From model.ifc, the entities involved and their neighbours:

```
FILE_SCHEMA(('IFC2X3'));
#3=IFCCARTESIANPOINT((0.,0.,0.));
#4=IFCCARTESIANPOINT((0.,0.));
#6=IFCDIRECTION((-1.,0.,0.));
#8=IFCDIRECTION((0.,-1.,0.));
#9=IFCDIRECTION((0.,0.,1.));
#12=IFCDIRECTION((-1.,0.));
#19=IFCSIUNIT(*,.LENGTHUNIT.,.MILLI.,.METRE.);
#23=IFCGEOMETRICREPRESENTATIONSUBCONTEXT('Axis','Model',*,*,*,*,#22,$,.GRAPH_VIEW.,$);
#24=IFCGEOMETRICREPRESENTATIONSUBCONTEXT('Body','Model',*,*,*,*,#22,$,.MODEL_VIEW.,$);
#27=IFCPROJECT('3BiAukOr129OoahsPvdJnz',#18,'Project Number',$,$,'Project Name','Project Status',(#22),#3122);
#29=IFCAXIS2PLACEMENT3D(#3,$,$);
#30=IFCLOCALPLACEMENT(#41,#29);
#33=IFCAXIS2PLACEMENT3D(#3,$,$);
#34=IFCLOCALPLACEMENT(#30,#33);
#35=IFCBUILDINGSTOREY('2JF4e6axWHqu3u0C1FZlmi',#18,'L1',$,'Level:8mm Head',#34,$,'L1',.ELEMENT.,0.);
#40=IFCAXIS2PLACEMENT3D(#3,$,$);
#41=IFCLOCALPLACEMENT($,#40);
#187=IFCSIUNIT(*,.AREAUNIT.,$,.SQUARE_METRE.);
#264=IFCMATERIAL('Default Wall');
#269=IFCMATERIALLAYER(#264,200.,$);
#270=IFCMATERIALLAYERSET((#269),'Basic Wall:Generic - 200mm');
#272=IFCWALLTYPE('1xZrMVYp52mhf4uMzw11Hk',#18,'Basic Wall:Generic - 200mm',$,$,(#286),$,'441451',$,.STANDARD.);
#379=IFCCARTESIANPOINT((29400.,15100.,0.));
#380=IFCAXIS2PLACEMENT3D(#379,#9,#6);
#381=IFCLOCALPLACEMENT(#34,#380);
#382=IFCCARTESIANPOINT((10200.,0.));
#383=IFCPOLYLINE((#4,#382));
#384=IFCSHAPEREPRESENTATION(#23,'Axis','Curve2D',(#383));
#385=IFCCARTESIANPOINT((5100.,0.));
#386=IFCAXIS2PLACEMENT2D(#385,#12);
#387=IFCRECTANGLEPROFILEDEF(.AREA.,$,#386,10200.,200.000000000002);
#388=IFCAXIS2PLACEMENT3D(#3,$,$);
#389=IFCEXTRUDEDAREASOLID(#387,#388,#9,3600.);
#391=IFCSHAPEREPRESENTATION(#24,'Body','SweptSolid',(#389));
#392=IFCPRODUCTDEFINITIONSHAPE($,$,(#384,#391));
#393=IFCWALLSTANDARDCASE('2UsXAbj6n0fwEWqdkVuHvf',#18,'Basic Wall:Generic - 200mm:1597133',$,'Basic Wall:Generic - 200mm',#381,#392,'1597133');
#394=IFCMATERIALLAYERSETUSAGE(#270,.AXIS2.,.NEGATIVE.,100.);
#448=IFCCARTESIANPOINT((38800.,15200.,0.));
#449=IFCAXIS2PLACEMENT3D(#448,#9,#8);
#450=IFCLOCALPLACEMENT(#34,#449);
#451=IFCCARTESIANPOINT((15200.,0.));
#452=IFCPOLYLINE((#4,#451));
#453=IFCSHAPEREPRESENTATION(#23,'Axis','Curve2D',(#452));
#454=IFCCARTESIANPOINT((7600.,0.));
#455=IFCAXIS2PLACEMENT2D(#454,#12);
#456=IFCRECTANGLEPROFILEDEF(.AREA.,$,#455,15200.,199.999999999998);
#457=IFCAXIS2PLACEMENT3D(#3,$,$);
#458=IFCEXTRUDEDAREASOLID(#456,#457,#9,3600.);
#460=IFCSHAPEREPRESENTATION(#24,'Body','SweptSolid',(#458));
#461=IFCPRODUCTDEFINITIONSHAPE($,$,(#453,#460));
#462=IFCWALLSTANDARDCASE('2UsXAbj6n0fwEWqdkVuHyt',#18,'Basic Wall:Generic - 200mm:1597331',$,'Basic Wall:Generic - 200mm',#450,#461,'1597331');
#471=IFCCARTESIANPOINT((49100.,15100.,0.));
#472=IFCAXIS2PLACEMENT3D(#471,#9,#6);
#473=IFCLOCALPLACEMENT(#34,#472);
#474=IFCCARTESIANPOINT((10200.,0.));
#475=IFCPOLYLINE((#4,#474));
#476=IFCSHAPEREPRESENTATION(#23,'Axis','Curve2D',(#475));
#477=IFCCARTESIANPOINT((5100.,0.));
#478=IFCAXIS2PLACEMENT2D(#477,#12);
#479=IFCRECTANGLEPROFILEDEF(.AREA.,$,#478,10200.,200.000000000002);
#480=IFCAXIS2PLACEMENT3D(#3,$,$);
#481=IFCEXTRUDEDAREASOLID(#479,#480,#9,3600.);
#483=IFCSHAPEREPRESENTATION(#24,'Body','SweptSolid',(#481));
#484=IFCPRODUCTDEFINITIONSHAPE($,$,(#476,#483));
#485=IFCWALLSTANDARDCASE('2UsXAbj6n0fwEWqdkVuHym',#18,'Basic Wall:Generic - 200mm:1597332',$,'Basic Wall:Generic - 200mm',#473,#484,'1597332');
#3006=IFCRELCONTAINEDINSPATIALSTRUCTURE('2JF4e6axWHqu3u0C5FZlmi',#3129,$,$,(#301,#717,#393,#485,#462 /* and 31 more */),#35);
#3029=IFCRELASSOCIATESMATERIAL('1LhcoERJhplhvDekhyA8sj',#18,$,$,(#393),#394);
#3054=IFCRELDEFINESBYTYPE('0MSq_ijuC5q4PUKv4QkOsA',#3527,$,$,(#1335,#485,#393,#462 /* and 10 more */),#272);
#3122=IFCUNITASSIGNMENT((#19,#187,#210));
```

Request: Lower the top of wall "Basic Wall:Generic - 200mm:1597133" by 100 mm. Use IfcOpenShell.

```python
import ifcopenshell
import ifcopenshell.geom
import ifcopenshell.util.representation
import ifcopenshell.util.shape

model = ifcopenshell.open("model.ifc")
settings = ifcopenshell.geom.settings()


def volume(element):
    """Net volume in cubic metres, openings subtracted."""
    shape = ifcopenshell.geom.create_shape(settings, element)
    return ifcopenshell.util.shape.get_volume(shape.geometry)


wall = model.by_id(393)
before = volume(wall)

body = ifcopenshell.util.representation.get_representation(wall, "Model", "Body")
solid = body.Items[0]
old_height = solid.Depth
solid.Depth -= 100.0
after = volume(wall)

print(f"height {old_height:g} -> {solid.Depth:g}, volume {before:.3f} -> {after:.3f} m3")

model.write("model-out.ifc")
```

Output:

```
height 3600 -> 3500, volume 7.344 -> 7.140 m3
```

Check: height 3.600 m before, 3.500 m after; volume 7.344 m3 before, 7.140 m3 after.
